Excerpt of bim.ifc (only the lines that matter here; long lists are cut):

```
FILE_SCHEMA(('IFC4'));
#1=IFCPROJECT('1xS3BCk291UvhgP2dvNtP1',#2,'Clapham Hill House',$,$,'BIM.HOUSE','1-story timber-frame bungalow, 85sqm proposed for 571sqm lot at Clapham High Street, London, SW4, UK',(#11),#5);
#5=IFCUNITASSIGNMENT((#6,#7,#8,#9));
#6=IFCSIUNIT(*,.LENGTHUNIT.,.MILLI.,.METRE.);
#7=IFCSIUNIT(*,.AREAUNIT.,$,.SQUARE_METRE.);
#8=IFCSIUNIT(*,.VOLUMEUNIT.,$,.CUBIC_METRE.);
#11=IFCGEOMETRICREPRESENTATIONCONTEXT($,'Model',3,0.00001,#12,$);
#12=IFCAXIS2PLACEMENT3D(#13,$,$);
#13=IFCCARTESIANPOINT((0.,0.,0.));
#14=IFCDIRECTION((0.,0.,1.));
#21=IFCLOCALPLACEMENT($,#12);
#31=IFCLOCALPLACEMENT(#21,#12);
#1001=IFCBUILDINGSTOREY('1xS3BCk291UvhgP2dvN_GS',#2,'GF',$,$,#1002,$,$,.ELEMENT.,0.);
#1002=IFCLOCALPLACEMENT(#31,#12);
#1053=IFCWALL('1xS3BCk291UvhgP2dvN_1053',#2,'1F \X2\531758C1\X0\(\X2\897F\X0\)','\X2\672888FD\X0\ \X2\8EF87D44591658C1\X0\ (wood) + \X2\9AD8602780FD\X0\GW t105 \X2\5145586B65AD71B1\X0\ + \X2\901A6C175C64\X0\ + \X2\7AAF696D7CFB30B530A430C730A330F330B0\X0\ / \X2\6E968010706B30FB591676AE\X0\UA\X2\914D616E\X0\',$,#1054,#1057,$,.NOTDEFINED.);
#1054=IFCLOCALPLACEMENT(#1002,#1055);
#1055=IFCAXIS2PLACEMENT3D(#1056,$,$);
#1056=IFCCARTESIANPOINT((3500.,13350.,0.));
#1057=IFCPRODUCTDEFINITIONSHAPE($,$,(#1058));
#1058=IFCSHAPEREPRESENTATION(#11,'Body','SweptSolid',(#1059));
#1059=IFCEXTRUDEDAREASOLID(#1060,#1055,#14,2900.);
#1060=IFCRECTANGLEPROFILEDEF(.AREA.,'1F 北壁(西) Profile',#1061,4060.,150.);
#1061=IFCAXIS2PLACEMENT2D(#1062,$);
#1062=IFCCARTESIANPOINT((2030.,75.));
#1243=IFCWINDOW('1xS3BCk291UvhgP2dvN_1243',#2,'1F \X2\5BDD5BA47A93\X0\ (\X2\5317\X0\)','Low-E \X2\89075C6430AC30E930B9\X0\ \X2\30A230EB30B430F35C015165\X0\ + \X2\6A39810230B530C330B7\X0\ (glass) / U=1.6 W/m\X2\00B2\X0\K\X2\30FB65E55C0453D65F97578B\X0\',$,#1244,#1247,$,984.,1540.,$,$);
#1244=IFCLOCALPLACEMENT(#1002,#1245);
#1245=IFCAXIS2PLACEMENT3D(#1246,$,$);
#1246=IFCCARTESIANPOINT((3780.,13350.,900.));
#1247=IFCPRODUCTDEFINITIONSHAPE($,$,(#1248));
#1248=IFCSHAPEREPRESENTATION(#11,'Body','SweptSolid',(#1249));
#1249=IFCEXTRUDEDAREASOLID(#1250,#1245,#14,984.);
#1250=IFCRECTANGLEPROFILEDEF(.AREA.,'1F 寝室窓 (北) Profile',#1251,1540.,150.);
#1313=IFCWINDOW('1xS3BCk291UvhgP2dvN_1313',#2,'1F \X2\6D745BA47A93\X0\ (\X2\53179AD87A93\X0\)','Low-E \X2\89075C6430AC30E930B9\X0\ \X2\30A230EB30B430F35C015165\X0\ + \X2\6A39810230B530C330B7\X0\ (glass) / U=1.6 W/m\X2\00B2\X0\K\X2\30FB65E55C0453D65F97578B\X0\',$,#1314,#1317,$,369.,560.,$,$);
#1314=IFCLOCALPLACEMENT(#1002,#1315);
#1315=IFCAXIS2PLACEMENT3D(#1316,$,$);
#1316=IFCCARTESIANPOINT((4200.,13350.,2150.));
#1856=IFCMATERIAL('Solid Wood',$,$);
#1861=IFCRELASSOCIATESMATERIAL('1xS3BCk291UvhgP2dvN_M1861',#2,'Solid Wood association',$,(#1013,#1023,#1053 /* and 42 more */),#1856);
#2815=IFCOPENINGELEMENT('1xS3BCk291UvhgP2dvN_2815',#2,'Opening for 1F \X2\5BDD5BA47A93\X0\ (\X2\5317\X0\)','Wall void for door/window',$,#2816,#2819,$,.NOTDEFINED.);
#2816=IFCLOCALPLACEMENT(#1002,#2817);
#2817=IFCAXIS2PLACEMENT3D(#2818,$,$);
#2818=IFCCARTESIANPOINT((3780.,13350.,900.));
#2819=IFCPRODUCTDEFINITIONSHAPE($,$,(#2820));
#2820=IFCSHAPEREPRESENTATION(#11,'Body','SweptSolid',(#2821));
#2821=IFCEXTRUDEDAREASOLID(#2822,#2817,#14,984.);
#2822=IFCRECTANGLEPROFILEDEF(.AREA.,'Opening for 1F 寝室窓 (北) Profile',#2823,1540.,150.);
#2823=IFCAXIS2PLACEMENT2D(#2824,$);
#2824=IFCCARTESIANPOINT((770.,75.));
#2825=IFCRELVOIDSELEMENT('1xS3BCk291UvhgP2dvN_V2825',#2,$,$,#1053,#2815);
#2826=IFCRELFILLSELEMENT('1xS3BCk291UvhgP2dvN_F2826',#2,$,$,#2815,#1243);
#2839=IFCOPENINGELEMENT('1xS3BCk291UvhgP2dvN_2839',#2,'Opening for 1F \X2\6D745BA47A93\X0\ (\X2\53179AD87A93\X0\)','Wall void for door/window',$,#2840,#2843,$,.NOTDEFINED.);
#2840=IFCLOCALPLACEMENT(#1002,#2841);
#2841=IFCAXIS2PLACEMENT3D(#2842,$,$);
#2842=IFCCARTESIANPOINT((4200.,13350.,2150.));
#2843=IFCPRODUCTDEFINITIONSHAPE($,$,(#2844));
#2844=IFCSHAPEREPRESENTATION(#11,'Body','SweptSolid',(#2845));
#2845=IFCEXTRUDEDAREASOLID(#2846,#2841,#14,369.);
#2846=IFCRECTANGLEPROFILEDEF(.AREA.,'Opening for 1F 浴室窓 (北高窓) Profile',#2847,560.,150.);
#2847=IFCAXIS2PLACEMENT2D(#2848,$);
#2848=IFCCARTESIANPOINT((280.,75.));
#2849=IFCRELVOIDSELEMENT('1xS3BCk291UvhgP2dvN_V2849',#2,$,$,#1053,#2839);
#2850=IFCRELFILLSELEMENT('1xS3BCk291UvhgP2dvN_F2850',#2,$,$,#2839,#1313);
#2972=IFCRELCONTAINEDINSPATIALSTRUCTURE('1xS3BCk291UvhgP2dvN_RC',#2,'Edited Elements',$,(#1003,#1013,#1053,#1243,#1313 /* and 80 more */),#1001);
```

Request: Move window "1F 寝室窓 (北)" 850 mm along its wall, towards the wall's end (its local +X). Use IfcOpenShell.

```python
import ifcopenshell
import ifcopenshell.api.geometry
import ifcopenshell.util.placement
import ifcopenshell.util.unit

model = ifcopenshell.open("bim.ifc")
unit_scale = ifcopenshell.util.unit.calculate_unit_scale(model)

window = model.by_guid("1xS3BCk291UvhgP2dvN_1243")
opening = window.FillsVoids[0].RelatingOpeningElement
wall = opening.VoidsElements[0].RelatingBuildingElement

wall_matrix = ifcopenshell.util.placement.get_local_placement(wall.ObjectPlacement)
shift = wall_matrix[:3, 0] * 0.85 / unit_scale
before = ifcopenshell.util.placement.get_local_placement(window.ObjectPlacement)[:3, 3].copy()

# The window is not placed relative to its opening, so move both.
for product in (opening, window):
    matrix = ifcopenshell.util.placement.get_local_placement(product.ObjectPlacement)
    matrix[:3, 3] += shift
    ifcopenshell.api.geometry.edit_object_placement(model, product=product, matrix=matrix, is_si=False)

after = ifcopenshell.util.placement.get_local_placement(window.ObjectPlacement)[:3, 3]
print("window moved by", (after - before).round(3) + 0.0)

model.write("bim_v2.ifc")
```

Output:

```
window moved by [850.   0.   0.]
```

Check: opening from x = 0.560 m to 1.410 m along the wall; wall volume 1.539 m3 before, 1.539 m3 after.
